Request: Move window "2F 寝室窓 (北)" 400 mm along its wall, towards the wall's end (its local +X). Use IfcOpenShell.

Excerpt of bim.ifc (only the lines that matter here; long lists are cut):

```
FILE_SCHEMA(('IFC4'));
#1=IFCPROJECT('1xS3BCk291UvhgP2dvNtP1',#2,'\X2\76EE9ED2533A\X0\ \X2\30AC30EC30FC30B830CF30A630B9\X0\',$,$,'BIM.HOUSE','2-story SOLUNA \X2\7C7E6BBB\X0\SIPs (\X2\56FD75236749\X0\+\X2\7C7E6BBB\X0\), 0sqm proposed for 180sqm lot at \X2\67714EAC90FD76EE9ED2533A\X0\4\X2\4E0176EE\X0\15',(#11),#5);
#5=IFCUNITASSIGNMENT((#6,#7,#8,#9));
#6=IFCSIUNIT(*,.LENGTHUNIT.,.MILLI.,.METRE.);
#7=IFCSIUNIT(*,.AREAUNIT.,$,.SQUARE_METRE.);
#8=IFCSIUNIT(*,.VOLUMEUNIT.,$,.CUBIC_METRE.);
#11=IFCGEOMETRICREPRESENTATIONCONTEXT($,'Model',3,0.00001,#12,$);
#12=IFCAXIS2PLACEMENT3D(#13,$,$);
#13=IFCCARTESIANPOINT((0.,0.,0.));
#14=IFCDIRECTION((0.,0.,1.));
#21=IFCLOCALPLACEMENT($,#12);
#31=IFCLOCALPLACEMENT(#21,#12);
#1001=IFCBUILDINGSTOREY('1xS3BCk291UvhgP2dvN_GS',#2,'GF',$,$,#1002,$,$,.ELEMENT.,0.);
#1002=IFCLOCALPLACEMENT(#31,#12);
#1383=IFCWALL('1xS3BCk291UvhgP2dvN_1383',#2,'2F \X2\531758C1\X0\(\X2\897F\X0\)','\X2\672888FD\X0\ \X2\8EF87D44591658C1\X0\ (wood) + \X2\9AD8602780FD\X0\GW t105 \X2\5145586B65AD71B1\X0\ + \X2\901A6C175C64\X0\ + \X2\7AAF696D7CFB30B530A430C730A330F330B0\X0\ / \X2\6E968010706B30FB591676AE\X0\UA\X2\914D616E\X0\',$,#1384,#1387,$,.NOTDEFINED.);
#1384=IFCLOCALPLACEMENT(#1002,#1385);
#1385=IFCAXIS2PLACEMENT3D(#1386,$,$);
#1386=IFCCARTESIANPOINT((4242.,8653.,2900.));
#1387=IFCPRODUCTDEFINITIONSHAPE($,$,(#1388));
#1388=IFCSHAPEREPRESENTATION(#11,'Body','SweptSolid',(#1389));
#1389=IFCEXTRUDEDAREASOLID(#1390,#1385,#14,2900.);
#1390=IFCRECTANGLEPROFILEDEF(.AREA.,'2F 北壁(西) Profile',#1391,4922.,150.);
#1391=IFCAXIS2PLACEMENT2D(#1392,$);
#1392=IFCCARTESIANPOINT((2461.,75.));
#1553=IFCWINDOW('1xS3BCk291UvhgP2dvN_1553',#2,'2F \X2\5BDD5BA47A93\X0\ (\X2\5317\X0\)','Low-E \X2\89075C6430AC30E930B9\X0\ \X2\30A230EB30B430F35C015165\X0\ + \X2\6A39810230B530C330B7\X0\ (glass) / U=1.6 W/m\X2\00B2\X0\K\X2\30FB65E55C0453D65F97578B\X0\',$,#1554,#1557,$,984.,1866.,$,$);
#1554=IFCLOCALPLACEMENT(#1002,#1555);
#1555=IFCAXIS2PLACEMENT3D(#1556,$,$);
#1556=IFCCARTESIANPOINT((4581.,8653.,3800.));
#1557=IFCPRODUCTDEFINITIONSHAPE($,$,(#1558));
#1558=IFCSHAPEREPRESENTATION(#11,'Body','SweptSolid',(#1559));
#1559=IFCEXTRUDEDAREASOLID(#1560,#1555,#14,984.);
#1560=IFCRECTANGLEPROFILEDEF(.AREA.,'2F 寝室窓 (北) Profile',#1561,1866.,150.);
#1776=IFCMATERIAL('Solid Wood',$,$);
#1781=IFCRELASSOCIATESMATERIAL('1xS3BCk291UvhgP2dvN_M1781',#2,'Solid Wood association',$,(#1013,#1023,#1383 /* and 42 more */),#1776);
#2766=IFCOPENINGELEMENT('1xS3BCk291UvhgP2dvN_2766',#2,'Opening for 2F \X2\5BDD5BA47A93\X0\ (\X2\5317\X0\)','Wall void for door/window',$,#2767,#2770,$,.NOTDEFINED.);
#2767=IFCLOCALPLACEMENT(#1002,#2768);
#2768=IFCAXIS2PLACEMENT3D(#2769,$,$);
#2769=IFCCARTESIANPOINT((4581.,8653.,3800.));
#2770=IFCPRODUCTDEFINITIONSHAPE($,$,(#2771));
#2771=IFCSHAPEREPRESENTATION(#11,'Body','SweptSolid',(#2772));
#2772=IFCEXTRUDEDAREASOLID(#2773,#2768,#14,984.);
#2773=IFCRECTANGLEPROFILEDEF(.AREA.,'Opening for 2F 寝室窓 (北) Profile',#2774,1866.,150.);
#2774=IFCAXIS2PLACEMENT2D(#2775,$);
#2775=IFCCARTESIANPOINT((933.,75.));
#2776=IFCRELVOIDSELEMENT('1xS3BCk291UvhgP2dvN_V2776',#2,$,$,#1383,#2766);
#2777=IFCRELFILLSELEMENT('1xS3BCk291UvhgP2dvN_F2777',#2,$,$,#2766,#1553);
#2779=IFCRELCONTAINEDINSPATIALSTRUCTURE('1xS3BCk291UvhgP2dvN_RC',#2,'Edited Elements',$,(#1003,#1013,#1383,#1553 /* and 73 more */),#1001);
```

```python
import ifcopenshell
import ifcopenshell.api.geometry
import ifcopenshell.util.placement
import ifcopenshell.util.unit

model = ifcopenshell.open("bim.ifc")
unit_scale = ifcopenshell.util.unit.calculate_unit_scale(model)

window = model.by_guid("1xS3BCk291UvhgP2dvN_1553")
opening = window.FillsVoids[0].RelatingOpeningElement
wall = opening.VoidsElements[0].RelatingBuildingElement

wall_matrix = ifcopenshell.util.placement.get_local_placement(wall.ObjectPlacement)
shift = wall_matrix[:3, 0] * 0.4 / unit_scale
before = ifcopenshell.util.placement.get_local_placement(window.ObjectPlacement)[:3, 3].copy()

# The window is not placed relative to its opening, so move both.
for product in (opening, window):
    matrix = ifcopenshell.util.placement.get_local_placement(product.ObjectPlacement)
    matrix[:3, 3] += shift
    ifcopenshell.api.geometry.edit_object_placement(model, product=product, matrix=matrix, is_si=False)

after = ifcopenshell.util.placement.get_local_placement(window.ObjectPlacement)[:3, 3]
print("window moved by", (after - before).round(3) + 0.0)

model.write("bim_updated.ifc")
```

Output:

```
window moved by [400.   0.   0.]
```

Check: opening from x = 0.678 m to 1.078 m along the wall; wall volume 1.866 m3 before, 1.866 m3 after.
